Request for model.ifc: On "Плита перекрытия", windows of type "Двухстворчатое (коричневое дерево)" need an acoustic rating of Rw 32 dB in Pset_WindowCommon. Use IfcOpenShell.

First a look at what the model holds.

```python
import ifcopenshell
import ifcopenshell.util.element

model = ifcopenshell.open("model.ifc")
print(model.schema)
storey = next(s for s in model.by_type("IfcBuildingStorey") if s.Name == "Плита перекрытия")
windows = [e for e in ifcopenshell.util.element.get_decomposition(storey) if e.is_a("IfcWindow")]
seen = {}
for e in windows:
    element_type = ifcopenshell.util.element.get_type(e)
    key = (element_type.Name if element_type != e and element_type else None, ifcopenshell.util.element.get_pset(e, "Pset_WindowCommon", "AcousticRating"))
    seen[key] = seen.get(key, 0) + 1
for (name, value), count in sorted(seen.items(), key=str):
    print(count, "x", name, "|", value)
```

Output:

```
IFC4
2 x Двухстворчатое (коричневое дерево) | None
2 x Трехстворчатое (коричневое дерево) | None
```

```python
import ifcopenshell
import ifcopenshell.api.pset
import ifcopenshell.util.element

model = ifcopenshell.open("model.ifc")

storey = next(s for s in model.by_type("IfcBuildingStorey") if s.Name == "Плита перекрытия")
windows = [e for e in ifcopenshell.util.element.get_decomposition(storey) if e.is_a("IfcWindow")]

count = 0
for e in windows:
    element_type = ifcopenshell.util.element.get_type(e)
    if element_type in (None, e) or element_type.Name != "Двухстворчатое (коричневое дерево)":
        continue
    # add_pset returns the element's existing set when there is one.
    pset = ifcopenshell.api.pset.add_pset(model, product=e, name="Pset_WindowCommon")
    ifcopenshell.api.pset.edit_pset(model, pset=pset, properties={"AcousticRating": "Rw 32 dB"})
    count += 1

print(count, "windows updated")

model.write("model_rev.ifc")
```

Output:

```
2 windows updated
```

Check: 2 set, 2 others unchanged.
